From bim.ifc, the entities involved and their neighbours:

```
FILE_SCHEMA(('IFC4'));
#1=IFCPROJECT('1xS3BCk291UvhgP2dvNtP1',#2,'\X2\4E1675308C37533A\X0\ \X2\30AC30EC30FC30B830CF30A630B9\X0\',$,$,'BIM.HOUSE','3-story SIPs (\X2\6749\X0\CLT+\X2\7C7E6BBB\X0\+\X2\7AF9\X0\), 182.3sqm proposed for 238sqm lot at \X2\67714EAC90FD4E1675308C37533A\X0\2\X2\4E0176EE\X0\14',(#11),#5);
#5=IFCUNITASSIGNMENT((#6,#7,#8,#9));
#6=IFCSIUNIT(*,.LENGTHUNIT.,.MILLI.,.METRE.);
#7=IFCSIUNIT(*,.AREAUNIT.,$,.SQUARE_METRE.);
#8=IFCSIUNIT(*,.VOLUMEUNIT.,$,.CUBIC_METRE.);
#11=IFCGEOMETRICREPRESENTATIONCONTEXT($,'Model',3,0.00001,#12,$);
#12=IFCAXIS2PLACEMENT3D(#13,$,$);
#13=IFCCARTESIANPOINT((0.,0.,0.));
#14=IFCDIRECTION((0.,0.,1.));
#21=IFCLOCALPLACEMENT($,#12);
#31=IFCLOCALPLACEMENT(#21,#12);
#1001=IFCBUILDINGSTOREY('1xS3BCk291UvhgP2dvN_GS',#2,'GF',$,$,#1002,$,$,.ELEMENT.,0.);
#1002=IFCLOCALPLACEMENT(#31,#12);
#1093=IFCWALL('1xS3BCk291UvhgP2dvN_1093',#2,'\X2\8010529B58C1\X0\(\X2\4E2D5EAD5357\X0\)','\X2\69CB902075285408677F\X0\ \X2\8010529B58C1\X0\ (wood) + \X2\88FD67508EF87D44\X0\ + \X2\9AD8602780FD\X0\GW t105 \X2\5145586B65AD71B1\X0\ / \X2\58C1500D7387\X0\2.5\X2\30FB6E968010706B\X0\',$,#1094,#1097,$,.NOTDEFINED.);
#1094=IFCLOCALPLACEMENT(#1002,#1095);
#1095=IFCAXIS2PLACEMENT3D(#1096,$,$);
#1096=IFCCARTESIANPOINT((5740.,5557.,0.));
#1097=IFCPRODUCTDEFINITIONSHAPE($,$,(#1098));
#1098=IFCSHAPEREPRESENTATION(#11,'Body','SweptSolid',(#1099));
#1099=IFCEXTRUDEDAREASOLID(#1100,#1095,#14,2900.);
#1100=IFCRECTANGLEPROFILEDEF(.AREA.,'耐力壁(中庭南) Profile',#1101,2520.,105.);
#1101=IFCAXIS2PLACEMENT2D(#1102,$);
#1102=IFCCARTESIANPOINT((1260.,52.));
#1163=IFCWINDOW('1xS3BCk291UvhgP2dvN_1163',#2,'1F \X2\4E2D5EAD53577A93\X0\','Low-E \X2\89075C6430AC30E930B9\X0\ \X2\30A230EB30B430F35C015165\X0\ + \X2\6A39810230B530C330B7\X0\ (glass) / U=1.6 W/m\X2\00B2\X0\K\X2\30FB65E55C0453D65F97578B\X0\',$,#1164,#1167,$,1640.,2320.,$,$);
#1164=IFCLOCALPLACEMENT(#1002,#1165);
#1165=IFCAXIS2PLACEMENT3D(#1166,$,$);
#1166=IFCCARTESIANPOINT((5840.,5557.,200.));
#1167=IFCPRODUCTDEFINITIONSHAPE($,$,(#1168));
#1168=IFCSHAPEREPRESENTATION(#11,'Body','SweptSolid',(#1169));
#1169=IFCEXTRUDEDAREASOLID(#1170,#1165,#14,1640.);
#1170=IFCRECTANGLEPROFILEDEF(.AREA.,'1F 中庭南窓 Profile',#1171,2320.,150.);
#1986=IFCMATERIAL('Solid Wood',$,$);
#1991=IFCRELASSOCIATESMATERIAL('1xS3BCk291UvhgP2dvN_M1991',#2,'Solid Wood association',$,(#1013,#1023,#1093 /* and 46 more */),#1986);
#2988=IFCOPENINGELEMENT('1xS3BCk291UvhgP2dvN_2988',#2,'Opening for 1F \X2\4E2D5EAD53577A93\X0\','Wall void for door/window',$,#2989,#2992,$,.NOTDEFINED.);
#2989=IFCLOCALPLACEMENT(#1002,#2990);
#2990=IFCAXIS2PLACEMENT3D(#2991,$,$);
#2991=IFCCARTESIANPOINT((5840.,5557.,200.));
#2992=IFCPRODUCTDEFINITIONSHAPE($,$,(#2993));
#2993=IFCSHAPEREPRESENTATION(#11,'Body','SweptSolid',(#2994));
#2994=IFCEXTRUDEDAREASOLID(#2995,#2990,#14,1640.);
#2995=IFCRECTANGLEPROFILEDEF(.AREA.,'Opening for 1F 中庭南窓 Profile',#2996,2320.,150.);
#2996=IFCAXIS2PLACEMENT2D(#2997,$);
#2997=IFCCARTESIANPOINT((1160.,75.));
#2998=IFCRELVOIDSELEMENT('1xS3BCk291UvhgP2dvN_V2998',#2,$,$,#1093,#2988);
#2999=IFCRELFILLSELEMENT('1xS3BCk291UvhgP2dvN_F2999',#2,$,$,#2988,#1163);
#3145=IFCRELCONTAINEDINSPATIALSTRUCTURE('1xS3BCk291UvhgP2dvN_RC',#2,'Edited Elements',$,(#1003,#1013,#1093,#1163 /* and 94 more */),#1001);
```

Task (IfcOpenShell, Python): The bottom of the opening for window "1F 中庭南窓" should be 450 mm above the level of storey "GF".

```python
import numpy as np
import ifcopenshell
import ifcopenshell.api.geometry
import ifcopenshell.geom
import ifcopenshell.util.element
import ifcopenshell.util.placement
import ifcopenshell.util.shape
import ifcopenshell.util.unit

model = ifcopenshell.open("bim.ifc")
unit_scale = ifcopenshell.util.unit.calculate_unit_scale(model)

window = model.by_guid("1xS3BCk291UvhgP2dvN_1163")
opening = window.FillsVoids[0].RelatingOpeningElement
storey = ifcopenshell.util.element.get_container(window, ifc_class="IfcBuildingStorey")
level = ifcopenshell.util.placement.get_local_placement(storey.ObjectPlacement)[2, 3]

# The opening's origin need not be at the sill, so measure its lowest point.
shape = ifcopenshell.geom.create_shape(ifcopenshell.geom.settings(), opening)
bottom = ifcopenshell.util.shape.get_shape_bottom_elevation(shape, shape.geometry) / unit_scale
dz = level + 450.0 - bottom

shift = np.array([0.0, 0.0, dz])
# The window is not placed relative to its opening, so move both.
for product in (opening, window):
    matrix = ifcopenshell.util.placement.get_local_placement(product.ObjectPlacement)
    matrix[:3, 3] += shift
    ifcopenshell.api.geometry.edit_object_placement(model, product=product, matrix=matrix, is_si=False)

print(f"moved by {dz * unit_scale:+.3f} m")

model.write("bim_v2.ifc")
```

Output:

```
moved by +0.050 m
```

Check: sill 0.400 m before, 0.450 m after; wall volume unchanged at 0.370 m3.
